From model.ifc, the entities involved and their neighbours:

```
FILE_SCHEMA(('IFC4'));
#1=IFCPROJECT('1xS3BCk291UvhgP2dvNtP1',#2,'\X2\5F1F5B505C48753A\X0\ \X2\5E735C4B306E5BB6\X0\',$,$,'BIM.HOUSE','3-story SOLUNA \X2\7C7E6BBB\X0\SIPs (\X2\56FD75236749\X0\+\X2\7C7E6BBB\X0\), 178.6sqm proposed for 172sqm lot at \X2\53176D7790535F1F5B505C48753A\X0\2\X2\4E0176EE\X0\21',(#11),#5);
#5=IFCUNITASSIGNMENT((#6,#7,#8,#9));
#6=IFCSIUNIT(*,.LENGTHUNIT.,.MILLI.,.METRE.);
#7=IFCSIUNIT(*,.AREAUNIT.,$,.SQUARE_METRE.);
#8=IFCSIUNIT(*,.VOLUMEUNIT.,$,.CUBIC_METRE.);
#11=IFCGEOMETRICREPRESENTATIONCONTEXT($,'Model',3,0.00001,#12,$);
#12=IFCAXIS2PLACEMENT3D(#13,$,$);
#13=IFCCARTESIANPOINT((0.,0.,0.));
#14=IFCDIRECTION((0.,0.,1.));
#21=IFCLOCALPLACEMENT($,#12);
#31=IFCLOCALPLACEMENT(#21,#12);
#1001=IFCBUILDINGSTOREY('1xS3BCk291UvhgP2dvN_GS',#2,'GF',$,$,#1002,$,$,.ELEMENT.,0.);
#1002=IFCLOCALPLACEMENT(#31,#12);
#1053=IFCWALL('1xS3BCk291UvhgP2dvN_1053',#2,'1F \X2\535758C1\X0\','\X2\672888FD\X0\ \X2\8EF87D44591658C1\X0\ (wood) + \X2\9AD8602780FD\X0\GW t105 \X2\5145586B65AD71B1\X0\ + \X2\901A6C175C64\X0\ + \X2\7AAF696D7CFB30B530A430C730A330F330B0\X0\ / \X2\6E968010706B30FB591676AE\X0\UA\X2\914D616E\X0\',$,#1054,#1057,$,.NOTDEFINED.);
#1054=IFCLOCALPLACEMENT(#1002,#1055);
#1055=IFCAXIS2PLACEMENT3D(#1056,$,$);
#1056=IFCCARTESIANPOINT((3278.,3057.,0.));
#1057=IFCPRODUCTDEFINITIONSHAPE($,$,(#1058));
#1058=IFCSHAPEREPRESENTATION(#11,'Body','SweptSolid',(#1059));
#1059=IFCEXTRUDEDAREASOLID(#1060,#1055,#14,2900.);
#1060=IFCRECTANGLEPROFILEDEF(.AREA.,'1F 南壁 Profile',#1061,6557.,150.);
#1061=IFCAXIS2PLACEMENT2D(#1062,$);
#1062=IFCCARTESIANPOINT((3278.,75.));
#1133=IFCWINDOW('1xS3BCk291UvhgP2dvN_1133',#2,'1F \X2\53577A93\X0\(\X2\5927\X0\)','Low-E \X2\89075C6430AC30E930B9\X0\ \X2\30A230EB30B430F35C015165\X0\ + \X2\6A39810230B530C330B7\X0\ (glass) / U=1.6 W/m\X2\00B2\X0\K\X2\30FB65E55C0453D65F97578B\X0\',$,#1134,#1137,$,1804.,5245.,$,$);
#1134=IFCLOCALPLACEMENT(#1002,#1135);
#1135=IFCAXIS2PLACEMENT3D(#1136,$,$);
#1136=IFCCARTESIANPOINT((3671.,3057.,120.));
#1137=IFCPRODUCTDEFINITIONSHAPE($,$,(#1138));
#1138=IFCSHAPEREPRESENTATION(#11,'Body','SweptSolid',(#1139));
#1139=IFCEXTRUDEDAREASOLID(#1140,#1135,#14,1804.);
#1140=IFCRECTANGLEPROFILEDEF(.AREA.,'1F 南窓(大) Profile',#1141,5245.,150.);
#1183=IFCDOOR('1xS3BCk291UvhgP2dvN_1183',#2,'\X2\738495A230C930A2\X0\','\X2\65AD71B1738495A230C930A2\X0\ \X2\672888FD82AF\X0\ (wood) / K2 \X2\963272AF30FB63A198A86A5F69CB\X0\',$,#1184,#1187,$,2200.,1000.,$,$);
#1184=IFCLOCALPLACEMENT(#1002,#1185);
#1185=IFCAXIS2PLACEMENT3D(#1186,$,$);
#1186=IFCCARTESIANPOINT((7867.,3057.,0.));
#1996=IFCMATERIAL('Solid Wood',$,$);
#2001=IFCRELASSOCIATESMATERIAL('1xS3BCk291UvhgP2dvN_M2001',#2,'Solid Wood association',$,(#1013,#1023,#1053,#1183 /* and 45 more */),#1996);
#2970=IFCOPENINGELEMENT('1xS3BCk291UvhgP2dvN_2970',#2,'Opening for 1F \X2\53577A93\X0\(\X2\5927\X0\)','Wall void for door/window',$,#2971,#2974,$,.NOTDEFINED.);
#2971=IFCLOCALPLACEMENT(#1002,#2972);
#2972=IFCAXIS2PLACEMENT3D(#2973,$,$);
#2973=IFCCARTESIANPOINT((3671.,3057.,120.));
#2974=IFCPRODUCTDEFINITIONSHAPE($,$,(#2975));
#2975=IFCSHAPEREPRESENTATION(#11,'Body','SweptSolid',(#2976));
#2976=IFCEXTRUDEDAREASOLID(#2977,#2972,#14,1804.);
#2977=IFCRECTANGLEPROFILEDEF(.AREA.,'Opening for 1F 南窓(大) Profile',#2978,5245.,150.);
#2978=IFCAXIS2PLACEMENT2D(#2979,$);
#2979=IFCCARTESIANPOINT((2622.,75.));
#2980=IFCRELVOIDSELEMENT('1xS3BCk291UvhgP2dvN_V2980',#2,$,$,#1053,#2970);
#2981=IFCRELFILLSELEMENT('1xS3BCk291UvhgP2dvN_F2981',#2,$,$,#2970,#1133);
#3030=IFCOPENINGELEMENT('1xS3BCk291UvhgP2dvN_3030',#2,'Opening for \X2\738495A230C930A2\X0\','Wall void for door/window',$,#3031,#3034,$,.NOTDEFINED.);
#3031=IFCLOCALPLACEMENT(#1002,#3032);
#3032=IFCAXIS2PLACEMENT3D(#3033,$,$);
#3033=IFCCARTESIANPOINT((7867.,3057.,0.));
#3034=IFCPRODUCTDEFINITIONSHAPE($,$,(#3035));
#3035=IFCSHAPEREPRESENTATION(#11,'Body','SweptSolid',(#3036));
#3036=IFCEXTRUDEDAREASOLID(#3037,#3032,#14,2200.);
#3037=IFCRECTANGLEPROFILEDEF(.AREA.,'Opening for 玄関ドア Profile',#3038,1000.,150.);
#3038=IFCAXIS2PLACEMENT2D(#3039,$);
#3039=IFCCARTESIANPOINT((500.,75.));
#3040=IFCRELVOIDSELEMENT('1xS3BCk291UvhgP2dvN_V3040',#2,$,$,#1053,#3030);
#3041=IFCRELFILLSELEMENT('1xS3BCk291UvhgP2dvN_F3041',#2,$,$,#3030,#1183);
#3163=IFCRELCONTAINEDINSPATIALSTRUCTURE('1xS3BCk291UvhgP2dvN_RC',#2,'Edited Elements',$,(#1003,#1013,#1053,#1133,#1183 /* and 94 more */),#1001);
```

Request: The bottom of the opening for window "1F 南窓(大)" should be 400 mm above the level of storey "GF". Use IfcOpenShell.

```python
import numpy as np
import ifcopenshell
import ifcopenshell.api.geometry
import ifcopenshell.geom
import ifcopenshell.util.element
import ifcopenshell.util.placement
import ifcopenshell.util.shape
import ifcopenshell.util.unit

model = ifcopenshell.open("model.ifc")
unit_scale = ifcopenshell.util.unit.calculate_unit_scale(model)

window = model.by_guid("1xS3BCk291UvhgP2dvN_1133")
opening = window.FillsVoids[0].RelatingOpeningElement
storey = ifcopenshell.util.element.get_container(window, ifc_class="IfcBuildingStorey")
level = ifcopenshell.util.placement.get_local_placement(storey.ObjectPlacement)[2, 3]

# The opening's origin need not be at the sill, so measure its lowest point.
shape = ifcopenshell.geom.create_shape(ifcopenshell.geom.settings(), opening)
bottom = ifcopenshell.util.shape.get_shape_bottom_elevation(shape, shape.geometry) / unit_scale
dz = level + 400.0 - bottom

shift = np.array([0.0, 0.0, dz])
# The window is not placed relative to its opening, so move both.
for product in (opening, window):
    matrix = ifcopenshell.util.placement.get_local_placement(product.ObjectPlacement)
    matrix[:3, 3] += shift
    ifcopenshell.api.geometry.edit_object_placement(model, product=product, matrix=matrix, is_si=False)

print(f"moved by {dz * unit_scale:+.3f} m")

model.write("model_rev.ifc")
```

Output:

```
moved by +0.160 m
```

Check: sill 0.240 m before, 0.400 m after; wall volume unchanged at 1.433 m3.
